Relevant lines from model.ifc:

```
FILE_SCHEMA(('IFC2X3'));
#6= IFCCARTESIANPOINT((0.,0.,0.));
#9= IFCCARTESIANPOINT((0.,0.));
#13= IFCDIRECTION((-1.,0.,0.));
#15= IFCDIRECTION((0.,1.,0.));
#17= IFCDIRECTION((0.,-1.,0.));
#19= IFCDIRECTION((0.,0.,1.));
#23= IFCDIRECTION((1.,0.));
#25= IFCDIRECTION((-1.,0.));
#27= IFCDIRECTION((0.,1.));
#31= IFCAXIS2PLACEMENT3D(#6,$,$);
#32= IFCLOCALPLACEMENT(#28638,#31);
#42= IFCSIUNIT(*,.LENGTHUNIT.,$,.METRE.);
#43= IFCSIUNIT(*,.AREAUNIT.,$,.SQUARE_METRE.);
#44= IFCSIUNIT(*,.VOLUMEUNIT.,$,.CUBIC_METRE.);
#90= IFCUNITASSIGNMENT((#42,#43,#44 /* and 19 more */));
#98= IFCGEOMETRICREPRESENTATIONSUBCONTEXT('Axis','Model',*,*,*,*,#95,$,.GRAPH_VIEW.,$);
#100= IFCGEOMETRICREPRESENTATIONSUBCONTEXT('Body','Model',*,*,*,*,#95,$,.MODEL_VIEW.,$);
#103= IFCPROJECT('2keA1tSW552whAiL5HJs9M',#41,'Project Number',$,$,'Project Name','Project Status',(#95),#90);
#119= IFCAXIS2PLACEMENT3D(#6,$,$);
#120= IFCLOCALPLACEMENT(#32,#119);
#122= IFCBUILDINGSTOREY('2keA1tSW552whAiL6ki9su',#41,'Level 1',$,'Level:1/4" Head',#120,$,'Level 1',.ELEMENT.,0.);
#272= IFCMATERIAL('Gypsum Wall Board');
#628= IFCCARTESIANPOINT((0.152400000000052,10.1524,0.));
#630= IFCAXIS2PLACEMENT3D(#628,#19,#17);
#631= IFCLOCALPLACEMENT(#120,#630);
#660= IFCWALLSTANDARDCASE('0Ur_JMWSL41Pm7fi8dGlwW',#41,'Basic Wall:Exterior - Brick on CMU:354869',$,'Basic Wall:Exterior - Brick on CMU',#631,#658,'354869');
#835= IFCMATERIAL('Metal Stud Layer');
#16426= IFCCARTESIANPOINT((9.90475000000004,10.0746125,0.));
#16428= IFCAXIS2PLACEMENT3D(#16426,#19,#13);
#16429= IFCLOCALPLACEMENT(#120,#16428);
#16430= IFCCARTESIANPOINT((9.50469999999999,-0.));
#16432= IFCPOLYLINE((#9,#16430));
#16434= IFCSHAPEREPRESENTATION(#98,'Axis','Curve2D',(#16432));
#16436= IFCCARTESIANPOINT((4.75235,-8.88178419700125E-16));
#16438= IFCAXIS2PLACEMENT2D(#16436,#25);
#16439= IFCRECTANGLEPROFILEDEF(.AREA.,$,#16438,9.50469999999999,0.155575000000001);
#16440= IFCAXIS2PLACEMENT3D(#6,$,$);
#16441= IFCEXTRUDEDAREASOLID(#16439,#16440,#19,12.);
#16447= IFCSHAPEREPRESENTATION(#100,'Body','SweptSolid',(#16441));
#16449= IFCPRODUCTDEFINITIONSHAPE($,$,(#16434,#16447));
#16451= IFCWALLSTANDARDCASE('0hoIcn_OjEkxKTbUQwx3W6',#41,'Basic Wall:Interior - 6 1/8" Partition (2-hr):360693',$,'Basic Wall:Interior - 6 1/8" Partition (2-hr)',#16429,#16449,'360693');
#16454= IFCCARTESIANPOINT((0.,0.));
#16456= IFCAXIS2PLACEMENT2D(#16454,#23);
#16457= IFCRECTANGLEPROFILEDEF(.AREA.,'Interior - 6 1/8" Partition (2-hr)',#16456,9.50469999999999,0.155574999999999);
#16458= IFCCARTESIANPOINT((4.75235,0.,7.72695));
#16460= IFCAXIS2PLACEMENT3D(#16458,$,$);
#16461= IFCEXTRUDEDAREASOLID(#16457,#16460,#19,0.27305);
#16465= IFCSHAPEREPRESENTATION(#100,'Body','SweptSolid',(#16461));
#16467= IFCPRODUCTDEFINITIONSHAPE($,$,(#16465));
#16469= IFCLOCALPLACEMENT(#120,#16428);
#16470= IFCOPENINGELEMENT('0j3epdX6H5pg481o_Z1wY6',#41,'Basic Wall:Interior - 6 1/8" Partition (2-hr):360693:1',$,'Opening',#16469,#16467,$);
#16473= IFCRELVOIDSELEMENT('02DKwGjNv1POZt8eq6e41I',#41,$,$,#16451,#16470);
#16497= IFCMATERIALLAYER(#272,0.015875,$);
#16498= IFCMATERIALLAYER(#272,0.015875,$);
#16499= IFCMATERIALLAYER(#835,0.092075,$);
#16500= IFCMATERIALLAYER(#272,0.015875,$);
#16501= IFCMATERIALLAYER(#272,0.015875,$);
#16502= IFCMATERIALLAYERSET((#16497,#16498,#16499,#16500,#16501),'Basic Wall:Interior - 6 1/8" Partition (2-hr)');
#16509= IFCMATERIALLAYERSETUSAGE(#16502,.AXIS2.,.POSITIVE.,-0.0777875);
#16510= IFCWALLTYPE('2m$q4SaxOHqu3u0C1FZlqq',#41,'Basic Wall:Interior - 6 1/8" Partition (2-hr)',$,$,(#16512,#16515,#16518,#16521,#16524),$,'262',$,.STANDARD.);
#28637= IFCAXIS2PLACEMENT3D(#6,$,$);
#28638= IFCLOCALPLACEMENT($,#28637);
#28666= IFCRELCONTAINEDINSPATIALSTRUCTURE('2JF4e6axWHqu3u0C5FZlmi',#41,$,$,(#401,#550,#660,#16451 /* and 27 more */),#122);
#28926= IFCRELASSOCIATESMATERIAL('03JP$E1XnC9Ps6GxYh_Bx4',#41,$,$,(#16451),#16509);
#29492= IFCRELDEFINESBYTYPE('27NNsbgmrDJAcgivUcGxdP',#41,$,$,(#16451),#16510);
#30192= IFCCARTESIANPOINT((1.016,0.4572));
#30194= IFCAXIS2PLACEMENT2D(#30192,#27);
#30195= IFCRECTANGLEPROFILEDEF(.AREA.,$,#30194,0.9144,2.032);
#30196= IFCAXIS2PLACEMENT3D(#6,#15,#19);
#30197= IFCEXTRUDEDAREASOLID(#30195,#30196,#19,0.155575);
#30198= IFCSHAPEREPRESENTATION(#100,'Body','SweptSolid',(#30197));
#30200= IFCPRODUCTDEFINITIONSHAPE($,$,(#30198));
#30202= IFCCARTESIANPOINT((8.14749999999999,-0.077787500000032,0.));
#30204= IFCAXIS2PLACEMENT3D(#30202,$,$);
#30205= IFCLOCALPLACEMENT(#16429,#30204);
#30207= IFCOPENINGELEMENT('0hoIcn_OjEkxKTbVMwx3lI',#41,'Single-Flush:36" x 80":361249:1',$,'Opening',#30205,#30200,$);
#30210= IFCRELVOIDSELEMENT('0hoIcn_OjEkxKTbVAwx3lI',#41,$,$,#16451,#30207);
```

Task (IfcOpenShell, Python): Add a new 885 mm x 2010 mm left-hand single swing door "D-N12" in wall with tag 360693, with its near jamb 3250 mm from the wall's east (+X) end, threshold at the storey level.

```python
import numpy as np
import ifcopenshell
import ifcopenshell.api.feature
import ifcopenshell.api.geometry
import ifcopenshell.api.root
import ifcopenshell.api.spatial
import ifcopenshell.api.type
import ifcopenshell.geom
import ifcopenshell.util.element
import ifcopenshell.util.placement
import ifcopenshell.util.representation
import ifcopenshell.util.shape
import ifcopenshell.util.unit

model = ifcopenshell.open("model.ifc")
unit_scale = ifcopenshell.util.unit.calculate_unit_scale(model)
settings = ifcopenshell.geom.settings()


def volume(element):
    """Net volume in cubic metres, openings subtracted."""
    shape = ifcopenshell.geom.create_shape(settings, element)
    return ifcopenshell.util.shape.get_volume(shape.geometry)


wall = model.by_id(16451)
storey = ifcopenshell.util.element.get_container(wall, ifc_class="IfcBuildingStorey")
context = ifcopenshell.util.representation.get_context(model, "Model", "Body", "MODEL_VIEW")
before = volume(wall)

width, height, from_end, sill = 0.885, 2.01, 3.25, 0.0  # metres

# The wall runs along its own X axis, and the end named is its -X end.
wall_shape = ifcopenshell.geom.create_shape(settings, wall)
x, y, z = ifcopenshell.util.shape.get_vertices(wall_shape.geometry).T
start = x.min() + from_end
face, thickness = float(y.min()), float(y.max() - y.min())
wall_matrix = ifcopenshell.util.placement.get_local_placement(wall.ObjectPlacement)
level = ifcopenshell.util.placement.get_local_placement(storey.ObjectPlacement)[2, 3]


def in_wall(x, y):
    """Placement at x, y metres in the wall's axes, at sill height."""
    matrix = wall_matrix.copy()
    matrix[:, 3] = wall_matrix @ np.array([x / unit_scale, y / unit_scale, 0.0, 1.0])
    matrix[2, 3] = level + sill / unit_scale
    return matrix


# Opening: a box that overshoots both wall faces by 50 mm.
opening = ifcopenshell.api.root.create_entity(model, ifc_class="IfcOpeningElement")
box = ifcopenshell.api.geometry.add_wall_representation(
    model, context=context, length=width, height=height, thickness=thickness + 0.1
)
ifcopenshell.api.geometry.assign_representation(model, product=opening, representation=box)
ifcopenshell.api.geometry.edit_object_placement(model, product=opening, matrix=in_wall(start, face - 0.05), is_si=False)
ifcopenshell.api.feature.add_feature(model, feature=opening, element=wall)

door = ifcopenshell.api.root.create_entity(model, ifc_class="IfcDoor", name="D-N12")
door.OverallWidth, door.OverallHeight = width / unit_scale, height / unit_scale
body = ifcopenshell.api.geometry.add_door_representation(
    model,
    context=context,
    overall_width=door.OverallWidth,
    overall_height=door.OverallHeight,
    operation_type="SINGLE_SWING_LEFT",
    lining_properties={"LiningDepth": thickness / unit_scale, "ThresholdDepth": thickness / unit_scale},
)
ifcopenshell.api.geometry.assign_representation(model, product=door, representation=body)
ifcopenshell.api.spatial.assign_container(model, products=[door], relating_structure=storey)
fills = ifcopenshell.api.feature.add_filling(model, opening=opening, element=door)
fills.OwnerHistory = door.OwnerHistory  # required in IFC2X3

# IFC2X3 keeps the operation on the door style.
style = ifcopenshell.api.root.create_entity(model, ifc_class="IfcDoorStyle", name="D-N12")
style.OperationType, style.ConstructionType = "SINGLE_SWING_LEFT", "NOTDEFINED"
style.ParameterTakesPrecedence = style.Sizeable = False
ifcopenshell.api.type.assign_type(model, related_objects=[door], relating_type=style)

# The lining spans the wall, so the door starts at the wall face.
ifcopenshell.api.geometry.edit_object_placement(model, product=door, matrix=in_wall(start, face), is_si=False)

after = volume(wall)

print(f"wall volume {before:.3f} -> {after:.3f} m3")

model.write("model_rev.ifc")
```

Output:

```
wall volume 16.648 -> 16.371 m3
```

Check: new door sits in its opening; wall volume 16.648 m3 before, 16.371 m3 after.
